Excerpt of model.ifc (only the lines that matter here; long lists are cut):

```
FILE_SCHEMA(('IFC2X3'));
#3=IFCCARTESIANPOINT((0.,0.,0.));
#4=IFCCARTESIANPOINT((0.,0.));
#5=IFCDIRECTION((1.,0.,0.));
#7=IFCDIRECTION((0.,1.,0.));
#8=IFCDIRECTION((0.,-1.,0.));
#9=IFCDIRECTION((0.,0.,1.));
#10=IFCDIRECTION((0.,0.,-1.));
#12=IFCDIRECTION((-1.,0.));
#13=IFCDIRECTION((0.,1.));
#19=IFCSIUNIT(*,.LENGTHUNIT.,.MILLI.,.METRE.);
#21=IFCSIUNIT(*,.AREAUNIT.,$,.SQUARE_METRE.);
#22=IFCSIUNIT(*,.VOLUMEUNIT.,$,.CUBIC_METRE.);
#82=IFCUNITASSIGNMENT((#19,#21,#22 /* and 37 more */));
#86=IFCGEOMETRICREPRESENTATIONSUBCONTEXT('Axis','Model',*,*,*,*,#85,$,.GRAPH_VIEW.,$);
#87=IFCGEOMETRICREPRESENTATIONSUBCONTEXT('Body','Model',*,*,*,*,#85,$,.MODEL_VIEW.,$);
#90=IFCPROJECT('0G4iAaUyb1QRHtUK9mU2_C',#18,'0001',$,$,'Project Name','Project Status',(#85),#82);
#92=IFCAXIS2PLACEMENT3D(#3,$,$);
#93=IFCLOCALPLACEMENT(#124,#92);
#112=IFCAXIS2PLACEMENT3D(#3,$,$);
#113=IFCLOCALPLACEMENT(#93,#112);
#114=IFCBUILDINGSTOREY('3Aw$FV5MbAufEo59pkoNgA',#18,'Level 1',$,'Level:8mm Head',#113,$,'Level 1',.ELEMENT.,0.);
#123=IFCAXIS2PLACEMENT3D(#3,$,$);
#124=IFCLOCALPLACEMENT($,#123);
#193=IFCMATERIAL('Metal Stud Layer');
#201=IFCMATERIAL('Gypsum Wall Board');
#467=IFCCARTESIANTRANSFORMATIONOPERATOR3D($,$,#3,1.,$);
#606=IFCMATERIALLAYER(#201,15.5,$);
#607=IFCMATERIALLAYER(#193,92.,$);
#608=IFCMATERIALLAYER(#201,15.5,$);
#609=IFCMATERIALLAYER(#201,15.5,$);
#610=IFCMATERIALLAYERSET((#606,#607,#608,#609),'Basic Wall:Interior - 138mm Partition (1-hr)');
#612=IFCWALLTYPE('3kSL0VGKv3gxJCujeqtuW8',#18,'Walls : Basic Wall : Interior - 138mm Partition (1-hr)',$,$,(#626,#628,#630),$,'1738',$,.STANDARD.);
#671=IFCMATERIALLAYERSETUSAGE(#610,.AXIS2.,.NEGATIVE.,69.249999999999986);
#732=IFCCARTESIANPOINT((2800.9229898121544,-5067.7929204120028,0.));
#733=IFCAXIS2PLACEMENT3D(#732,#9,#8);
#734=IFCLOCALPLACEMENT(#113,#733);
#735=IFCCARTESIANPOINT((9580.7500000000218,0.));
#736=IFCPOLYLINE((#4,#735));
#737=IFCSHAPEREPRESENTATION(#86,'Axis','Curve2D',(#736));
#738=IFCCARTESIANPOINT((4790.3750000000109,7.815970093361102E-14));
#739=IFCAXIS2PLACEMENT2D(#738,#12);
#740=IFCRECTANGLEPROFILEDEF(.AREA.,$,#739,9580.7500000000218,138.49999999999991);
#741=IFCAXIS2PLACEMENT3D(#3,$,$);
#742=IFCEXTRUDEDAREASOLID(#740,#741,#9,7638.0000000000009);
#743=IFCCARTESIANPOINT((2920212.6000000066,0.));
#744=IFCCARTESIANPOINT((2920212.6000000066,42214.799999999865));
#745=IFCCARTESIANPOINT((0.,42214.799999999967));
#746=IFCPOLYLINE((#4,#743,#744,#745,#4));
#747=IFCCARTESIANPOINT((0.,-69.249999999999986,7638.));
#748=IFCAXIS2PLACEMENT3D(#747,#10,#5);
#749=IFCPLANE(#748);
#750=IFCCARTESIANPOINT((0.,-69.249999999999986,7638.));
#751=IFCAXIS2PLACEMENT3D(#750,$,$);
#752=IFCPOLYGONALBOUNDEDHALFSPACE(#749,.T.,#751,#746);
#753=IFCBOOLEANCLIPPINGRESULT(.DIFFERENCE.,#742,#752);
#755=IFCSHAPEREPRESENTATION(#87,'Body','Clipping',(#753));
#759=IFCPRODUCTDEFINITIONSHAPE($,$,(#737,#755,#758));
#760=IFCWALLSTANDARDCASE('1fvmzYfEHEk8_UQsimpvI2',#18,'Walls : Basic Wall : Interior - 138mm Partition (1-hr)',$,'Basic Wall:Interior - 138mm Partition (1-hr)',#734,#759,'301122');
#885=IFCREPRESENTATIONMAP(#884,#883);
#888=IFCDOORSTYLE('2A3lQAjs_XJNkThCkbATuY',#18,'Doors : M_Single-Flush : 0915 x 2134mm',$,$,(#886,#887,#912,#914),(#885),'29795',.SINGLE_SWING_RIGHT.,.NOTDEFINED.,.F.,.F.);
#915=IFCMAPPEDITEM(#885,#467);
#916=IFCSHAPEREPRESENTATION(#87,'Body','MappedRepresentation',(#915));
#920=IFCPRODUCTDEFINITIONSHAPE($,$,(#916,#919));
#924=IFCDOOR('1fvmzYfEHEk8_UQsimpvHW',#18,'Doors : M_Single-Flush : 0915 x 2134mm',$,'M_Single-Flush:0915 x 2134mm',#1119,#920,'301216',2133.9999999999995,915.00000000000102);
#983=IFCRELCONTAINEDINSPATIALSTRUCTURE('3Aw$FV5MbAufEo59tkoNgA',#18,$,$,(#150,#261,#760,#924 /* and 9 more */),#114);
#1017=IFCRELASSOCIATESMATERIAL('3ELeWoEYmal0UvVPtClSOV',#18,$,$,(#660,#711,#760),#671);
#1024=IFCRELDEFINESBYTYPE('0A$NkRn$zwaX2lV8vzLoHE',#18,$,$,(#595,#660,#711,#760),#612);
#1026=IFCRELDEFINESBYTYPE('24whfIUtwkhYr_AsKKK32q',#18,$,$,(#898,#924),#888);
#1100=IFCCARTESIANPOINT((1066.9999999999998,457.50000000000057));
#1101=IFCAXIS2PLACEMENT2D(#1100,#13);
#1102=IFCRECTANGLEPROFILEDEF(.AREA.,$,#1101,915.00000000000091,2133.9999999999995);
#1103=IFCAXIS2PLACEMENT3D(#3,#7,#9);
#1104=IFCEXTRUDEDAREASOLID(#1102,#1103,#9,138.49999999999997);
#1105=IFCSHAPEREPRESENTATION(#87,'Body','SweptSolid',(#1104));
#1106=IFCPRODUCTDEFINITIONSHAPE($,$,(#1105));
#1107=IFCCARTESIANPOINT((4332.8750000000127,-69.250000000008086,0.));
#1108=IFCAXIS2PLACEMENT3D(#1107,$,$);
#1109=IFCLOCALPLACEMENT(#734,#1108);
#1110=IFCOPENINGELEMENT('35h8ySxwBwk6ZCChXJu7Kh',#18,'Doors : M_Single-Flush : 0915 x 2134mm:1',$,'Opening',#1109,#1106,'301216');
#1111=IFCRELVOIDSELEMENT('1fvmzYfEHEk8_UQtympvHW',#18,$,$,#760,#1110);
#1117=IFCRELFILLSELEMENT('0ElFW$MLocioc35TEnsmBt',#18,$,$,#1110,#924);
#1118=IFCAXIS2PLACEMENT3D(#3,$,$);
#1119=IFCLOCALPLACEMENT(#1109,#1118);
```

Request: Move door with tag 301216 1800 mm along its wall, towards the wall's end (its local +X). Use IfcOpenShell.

```python
import ifcopenshell
import ifcopenshell.api.geometry
import ifcopenshell.util.placement
import ifcopenshell.util.unit

model = ifcopenshell.open("model.ifc")
unit_scale = ifcopenshell.util.unit.calculate_unit_scale(model)

door = model.by_guid("1fvmzYfEHEk8_UQsimpvHW")
opening = door.FillsVoids[0].RelatingOpeningElement
wall = opening.VoidsElements[0].RelatingBuildingElement

wall_matrix = ifcopenshell.util.placement.get_local_placement(wall.ObjectPlacement)
shift = wall_matrix[:3, 0] * 1.8 / unit_scale
before = ifcopenshell.util.placement.get_local_placement(door.ObjectPlacement)[:3, 3].copy()

# The door is placed relative to its opening, so it follows when the opening moves.
matrix = ifcopenshell.util.placement.get_local_placement(opening.ObjectPlacement)
matrix[:3, 3] += shift
ifcopenshell.api.geometry.edit_object_placement(
    model, product=opening, matrix=matrix, is_si=False, should_transform_children=True
)

after = ifcopenshell.util.placement.get_local_placement(door.ObjectPlacement)[:3, 3]
print("door moved by", (after - before).round(3) + 0.0)

model.write("model-out.ifc")
```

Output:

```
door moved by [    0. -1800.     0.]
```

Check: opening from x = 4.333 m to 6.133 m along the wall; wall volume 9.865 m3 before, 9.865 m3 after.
